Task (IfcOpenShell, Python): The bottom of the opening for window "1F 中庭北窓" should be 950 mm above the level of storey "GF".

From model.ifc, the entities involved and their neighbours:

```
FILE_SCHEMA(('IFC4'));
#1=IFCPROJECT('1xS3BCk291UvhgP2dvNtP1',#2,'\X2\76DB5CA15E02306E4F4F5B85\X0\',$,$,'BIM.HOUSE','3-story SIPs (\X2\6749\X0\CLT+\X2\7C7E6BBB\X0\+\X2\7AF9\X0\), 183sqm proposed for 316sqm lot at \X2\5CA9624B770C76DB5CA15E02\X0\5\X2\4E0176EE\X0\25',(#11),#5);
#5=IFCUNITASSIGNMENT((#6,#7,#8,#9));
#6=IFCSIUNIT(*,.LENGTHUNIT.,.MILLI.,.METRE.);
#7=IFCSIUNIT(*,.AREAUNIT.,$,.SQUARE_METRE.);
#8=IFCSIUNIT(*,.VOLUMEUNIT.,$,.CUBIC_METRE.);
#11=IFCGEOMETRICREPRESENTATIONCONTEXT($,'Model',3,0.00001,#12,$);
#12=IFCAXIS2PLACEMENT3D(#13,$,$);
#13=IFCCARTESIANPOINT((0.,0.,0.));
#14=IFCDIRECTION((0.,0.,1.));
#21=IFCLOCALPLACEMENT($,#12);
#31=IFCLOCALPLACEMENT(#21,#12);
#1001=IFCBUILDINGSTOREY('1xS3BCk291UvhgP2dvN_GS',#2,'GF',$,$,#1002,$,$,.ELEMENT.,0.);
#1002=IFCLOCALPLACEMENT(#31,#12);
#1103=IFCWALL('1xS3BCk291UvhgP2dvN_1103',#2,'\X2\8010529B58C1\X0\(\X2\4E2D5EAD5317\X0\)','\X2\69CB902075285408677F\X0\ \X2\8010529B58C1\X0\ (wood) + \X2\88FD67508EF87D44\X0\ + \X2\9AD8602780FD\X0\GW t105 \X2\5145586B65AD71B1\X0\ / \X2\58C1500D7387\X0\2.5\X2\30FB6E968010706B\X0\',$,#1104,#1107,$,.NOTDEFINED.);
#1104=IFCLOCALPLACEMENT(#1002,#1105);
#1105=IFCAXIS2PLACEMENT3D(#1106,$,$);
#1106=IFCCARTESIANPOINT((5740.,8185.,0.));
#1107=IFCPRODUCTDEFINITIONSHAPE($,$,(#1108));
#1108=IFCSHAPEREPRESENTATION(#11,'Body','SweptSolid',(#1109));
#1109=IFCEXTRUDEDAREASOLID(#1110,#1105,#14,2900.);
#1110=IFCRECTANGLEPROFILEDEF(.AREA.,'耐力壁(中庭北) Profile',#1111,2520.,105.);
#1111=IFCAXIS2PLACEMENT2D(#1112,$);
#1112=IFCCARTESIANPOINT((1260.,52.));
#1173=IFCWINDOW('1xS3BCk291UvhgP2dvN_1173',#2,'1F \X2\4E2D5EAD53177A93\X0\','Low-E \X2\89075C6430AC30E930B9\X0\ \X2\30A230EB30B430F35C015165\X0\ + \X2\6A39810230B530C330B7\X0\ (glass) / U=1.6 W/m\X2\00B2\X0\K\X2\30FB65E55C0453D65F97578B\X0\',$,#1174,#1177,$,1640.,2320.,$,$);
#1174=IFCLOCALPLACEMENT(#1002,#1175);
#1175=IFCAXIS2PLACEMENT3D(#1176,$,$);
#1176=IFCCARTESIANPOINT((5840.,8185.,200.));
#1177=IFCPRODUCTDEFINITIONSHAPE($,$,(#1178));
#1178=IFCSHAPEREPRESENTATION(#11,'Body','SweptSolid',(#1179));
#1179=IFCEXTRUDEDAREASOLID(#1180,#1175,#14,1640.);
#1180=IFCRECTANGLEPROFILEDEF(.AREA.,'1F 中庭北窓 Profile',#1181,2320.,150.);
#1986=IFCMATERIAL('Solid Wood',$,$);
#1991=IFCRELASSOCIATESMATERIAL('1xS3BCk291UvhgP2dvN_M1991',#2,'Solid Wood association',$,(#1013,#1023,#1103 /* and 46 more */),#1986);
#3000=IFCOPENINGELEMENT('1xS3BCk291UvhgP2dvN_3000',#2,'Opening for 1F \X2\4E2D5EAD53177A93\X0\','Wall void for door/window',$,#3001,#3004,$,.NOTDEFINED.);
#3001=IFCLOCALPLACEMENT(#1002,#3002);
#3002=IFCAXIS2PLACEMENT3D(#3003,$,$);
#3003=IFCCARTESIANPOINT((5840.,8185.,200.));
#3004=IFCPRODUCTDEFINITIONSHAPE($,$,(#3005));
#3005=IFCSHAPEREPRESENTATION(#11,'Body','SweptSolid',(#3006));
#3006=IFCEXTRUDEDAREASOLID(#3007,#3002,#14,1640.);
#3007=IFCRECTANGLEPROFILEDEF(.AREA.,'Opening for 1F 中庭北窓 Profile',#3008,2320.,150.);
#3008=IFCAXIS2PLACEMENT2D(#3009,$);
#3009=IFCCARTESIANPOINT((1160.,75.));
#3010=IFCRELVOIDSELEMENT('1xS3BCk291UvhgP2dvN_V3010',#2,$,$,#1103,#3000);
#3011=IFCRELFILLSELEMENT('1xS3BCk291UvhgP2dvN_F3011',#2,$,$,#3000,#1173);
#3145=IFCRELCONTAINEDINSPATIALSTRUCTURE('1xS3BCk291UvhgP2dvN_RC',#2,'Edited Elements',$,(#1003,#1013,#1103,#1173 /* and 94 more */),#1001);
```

```python
import numpy as np
import ifcopenshell
import ifcopenshell.api.geometry
import ifcopenshell.geom
import ifcopenshell.util.element
import ifcopenshell.util.placement
import ifcopenshell.util.shape
import ifcopenshell.util.unit

model = ifcopenshell.open("model.ifc")
unit_scale = ifcopenshell.util.unit.calculate_unit_scale(model)

window = model.by_guid("1xS3BCk291UvhgP2dvN_1173")
opening = window.FillsVoids[0].RelatingOpeningElement
storey = ifcopenshell.util.element.get_container(window, ifc_class="IfcBuildingStorey")
level = ifcopenshell.util.placement.get_local_placement(storey.ObjectPlacement)[2, 3]

# The opening's origin need not be at the sill, so measure its lowest point.
shape = ifcopenshell.geom.create_shape(ifcopenshell.geom.settings(), opening)
bottom = ifcopenshell.util.shape.get_shape_bottom_elevation(shape, shape.geometry) / unit_scale
dz = level + 0.95 / unit_scale - bottom

shift = np.array([0.0, 0.0, dz])
# The window is not placed relative to its opening, so move both.
for product in (opening, window):
    matrix = ifcopenshell.util.placement.get_local_placement(product.ObjectPlacement)
    matrix[:3, 3] += shift
    ifcopenshell.api.geometry.edit_object_placement(model, product=product, matrix=matrix, is_si=False)

print(f"moved by {dz * unit_scale:+.3f} m")

model.write("model_v2.ifc")
```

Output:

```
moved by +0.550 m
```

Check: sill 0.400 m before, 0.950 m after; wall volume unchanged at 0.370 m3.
